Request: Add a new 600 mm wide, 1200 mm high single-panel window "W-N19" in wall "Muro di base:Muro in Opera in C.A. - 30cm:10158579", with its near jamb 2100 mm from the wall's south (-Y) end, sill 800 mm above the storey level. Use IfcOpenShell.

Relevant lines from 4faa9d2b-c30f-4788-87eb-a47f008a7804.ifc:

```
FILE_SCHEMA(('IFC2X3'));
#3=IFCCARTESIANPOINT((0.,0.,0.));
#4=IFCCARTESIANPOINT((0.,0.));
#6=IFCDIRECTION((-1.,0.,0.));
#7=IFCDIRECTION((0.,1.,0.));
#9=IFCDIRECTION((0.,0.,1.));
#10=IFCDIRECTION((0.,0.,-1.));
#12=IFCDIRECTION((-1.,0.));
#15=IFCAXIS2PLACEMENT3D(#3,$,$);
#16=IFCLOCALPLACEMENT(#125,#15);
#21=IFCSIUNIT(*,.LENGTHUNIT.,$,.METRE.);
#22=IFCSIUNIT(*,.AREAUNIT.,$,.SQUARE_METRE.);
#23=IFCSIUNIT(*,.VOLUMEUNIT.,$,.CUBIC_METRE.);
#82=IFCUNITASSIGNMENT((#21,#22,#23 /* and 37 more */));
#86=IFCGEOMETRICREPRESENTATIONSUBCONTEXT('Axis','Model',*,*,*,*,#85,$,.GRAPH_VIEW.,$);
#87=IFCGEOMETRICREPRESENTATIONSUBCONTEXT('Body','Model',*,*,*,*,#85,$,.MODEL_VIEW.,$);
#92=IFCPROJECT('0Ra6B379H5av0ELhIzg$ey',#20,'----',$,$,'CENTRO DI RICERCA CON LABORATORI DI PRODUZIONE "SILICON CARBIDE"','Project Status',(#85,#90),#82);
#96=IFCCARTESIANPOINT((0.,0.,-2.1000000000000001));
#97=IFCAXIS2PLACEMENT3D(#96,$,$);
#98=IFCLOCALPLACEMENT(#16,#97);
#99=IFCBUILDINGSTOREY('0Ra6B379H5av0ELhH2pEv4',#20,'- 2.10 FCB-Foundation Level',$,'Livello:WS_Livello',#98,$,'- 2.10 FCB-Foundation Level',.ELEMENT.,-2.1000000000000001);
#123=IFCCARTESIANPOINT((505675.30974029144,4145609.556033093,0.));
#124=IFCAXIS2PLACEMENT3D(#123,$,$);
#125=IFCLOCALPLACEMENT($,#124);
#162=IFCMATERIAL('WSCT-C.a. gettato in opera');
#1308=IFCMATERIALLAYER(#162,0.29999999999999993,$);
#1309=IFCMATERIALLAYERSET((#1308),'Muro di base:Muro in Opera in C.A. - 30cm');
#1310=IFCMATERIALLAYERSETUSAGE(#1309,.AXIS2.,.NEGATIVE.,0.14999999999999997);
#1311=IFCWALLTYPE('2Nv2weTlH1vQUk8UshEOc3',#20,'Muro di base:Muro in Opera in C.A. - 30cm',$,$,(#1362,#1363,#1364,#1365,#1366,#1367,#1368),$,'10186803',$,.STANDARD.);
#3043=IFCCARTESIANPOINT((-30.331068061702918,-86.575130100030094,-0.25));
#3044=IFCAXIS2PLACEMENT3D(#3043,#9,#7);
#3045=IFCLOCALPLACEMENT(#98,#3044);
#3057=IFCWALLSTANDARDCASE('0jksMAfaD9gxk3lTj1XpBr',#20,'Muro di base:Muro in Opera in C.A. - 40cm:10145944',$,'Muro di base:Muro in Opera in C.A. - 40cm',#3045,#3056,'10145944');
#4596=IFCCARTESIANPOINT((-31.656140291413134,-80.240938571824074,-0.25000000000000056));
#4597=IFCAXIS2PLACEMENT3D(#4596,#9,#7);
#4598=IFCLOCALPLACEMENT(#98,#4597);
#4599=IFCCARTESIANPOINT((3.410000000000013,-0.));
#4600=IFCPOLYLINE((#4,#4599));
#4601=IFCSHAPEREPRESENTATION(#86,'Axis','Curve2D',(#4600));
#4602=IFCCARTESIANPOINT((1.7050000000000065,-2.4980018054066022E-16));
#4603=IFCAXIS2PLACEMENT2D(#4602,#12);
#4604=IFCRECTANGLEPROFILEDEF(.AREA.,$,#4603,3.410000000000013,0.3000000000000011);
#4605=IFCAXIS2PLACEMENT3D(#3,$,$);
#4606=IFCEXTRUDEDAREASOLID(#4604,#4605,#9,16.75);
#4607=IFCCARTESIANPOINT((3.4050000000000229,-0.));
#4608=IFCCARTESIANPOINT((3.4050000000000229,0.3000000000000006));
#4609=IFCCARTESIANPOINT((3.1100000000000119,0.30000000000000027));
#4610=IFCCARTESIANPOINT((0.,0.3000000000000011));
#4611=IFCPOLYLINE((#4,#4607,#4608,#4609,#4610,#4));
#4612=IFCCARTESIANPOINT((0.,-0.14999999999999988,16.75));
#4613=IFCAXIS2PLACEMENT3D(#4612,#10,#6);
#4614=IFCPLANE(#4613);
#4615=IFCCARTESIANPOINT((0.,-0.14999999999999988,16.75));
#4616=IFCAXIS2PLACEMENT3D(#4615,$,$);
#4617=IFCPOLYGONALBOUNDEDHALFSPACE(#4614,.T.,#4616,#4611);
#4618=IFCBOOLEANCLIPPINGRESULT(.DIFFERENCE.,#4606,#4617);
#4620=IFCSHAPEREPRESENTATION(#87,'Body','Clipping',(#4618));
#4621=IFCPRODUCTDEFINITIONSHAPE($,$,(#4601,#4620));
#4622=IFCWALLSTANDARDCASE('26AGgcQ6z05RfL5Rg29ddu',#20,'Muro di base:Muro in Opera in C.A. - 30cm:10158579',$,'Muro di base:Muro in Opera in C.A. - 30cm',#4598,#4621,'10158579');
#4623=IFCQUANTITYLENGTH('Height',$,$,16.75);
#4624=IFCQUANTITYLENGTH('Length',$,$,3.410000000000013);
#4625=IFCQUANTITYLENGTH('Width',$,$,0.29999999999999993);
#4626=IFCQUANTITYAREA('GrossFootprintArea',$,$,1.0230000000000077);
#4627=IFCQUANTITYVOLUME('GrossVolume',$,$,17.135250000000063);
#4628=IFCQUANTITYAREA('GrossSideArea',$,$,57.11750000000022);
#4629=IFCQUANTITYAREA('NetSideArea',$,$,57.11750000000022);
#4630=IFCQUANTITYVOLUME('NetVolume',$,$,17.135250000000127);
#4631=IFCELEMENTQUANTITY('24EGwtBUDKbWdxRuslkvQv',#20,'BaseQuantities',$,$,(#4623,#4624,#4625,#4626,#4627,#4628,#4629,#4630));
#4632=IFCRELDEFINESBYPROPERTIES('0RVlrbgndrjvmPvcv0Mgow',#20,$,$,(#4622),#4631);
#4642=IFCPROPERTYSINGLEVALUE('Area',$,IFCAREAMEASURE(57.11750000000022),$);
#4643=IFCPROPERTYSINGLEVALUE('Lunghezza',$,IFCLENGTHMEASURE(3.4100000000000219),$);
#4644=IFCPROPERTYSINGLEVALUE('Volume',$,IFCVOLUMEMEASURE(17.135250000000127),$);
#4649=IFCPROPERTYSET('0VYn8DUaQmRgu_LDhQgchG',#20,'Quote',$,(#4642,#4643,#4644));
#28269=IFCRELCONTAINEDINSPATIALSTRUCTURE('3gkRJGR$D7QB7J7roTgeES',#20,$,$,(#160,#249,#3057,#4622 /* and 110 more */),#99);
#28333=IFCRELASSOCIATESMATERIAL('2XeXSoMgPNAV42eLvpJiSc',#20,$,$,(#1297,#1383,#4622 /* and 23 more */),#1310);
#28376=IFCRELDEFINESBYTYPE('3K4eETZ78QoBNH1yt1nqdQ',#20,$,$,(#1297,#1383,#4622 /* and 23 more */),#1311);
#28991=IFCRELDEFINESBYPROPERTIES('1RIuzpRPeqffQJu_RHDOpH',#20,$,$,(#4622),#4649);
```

```python
import numpy as np
import ifcopenshell
import ifcopenshell.api.feature
import ifcopenshell.api.geometry
import ifcopenshell.api.pset
import ifcopenshell.api.root
import ifcopenshell.api.spatial
import ifcopenshell.api.type
import ifcopenshell.geom
import ifcopenshell.util.element
import ifcopenshell.util.placement
import ifcopenshell.util.representation
import ifcopenshell.util.shape
import ifcopenshell.util.unit

model = ifcopenshell.open("4faa9d2b-c30f-4788-87eb-a47f008a7804.ifc")
unit_scale = ifcopenshell.util.unit.calculate_unit_scale(model)
area_scale = ifcopenshell.util.unit.calculate_unit_scale(model, "AREAUNIT")
volume_scale = ifcopenshell.util.unit.calculate_unit_scale(model, "VOLUMEUNIT")
settings = ifcopenshell.geom.settings()


def volume(element):
    """Net volume in cubic metres, openings subtracted."""
    shape = ifcopenshell.geom.create_shape(settings, element)
    return ifcopenshell.util.shape.get_volume(shape.geometry)


wall = model.by_id(4622)
storey = ifcopenshell.util.element.get_container(wall, ifc_class="IfcBuildingStorey")
context = ifcopenshell.util.representation.get_context(model, "Model", "Body", "MODEL_VIEW")
before = volume(wall)

width, height, from_end, sill = 0.6, 1.2, 2.1, 0.8  # metres

# The wall runs along its own X axis, and the end named is its -X end.
wall_shape = ifcopenshell.geom.create_shape(settings, wall)
x, y, z = ifcopenshell.util.shape.get_vertices(wall_shape.geometry).T
start = x.min() + from_end
face, thickness = float(y.min()), float(y.max() - y.min())
wall_matrix = ifcopenshell.util.placement.get_local_placement(wall.ObjectPlacement)
level = ifcopenshell.util.placement.get_local_placement(storey.ObjectPlacement)[2, 3]


def in_wall(x, y):
    """Placement at x, y metres in the wall's axes, at sill height."""
    matrix = wall_matrix.copy()
    matrix[:, 3] = wall_matrix @ np.array([x / unit_scale, y / unit_scale, 0.0, 1.0])
    matrix[2, 3] = level + sill / unit_scale
    return matrix


# Opening: a box that overshoots both wall faces by 50 mm.
opening = ifcopenshell.api.root.create_entity(model, ifc_class="IfcOpeningElement")
box = ifcopenshell.api.geometry.add_wall_representation(
    model, context=context, length=width, height=height, thickness=thickness + 0.1
)
ifcopenshell.api.geometry.assign_representation(model, product=opening, representation=box)
ifcopenshell.api.geometry.edit_object_placement(model, product=opening, matrix=in_wall(start, face - 0.05), is_si=False)
ifcopenshell.api.feature.add_feature(model, feature=opening, element=wall)

window = ifcopenshell.api.root.create_entity(model, ifc_class="IfcWindow", name="W-N19")
window.OverallWidth, window.OverallHeight = width / unit_scale, height / unit_scale
body = ifcopenshell.api.geometry.add_window_representation(
    model,
    context=context,
    overall_width=window.OverallWidth,
    overall_height=window.OverallHeight,
    partition_type="SINGLE_PANEL",
)
ifcopenshell.api.geometry.assign_representation(model, product=window, representation=body)
ifcopenshell.api.spatial.assign_container(model, products=[window], relating_structure=storey)
fills = ifcopenshell.api.feature.add_filling(model, opening=opening, element=window)
fills.OwnerHistory = window.OwnerHistory  # required in IFC2X3

# IFC2X3 keeps the operation on the window style.
style = ifcopenshell.api.root.create_entity(model, ifc_class="IfcWindowStyle", name="W-N19")
style.OperationType, style.ConstructionType = "SINGLE_PANEL", "NOTDEFINED"
style.ParameterTakesPrecedence = style.Sizeable = False
ifcopenshell.api.type.assign_type(model, related_objects=[window], relating_type=style)

# Centre the window in the wall's thickness.
ifcopenshell.api.geometry.edit_object_placement(model, product=window, matrix=in_wall(start, face), is_si=False)
window_shape = ifcopenshell.geom.create_shape(settings, window)
depth = ifcopenshell.util.shape.get_vertices(window_shape.geometry)[:, 1]
offset = face + thickness / 2 - (depth.min() + depth.max()) / 2
ifcopenshell.api.geometry.edit_object_placement(model, product=window, matrix=in_wall(start, offset), is_si=False)

after = volume(wall)

# Update the wall's stored quantities.
qto = model.by_id(ifcopenshell.util.element.get_pset(wall, "BaseQuantities", should_inherit=False)["id"])
ifcopenshell.api.pset.edit_qto(model, qto=qto, properties={
    "NetSideArea": after / thickness / area_scale,
    "NetVolume": after / volume_scale,
})
pset = model.by_id(ifcopenshell.util.element.get_pset(wall, "Quote", should_inherit=False)["id"])
ifcopenshell.api.pset.edit_pset(model, pset=pset, properties={
    "Area": model.create_entity("IfcAreaMeasure", after / thickness / area_scale),
    "Volume": model.create_entity("IfcVolumeMeasure", after / volume_scale),
})

print(f"wall volume {before:.3f} -> {after:.3f} m3")

model.write("4faa9d2b-c30f-4788-87eb-a47f008a7804_v2.ifc")
```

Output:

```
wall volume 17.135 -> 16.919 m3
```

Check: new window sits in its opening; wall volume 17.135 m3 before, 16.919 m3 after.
